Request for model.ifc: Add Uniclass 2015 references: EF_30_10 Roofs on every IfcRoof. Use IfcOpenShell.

First a look at what the model holds.

```python
import ifcopenshell

model = ifcopenshell.open("model.ifc")
print(model.schema)
print("classifications:", [c.Name for c in model.by_type("IfcClassification")])
for ifc_class in ("IfcDoor", "IfcRoof", "IfcStair", "IfcWall", "IfcWindow"):
    print(ifc_class, len(model.by_type(ifc_class)))
```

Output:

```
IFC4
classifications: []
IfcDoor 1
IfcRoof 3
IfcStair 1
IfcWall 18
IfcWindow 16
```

```python
import ifcopenshell
import ifcopenshell.api.classification

model = ifcopenshell.open("model.ifc")

system = ifcopenshell.api.classification.add_classification(model, classification="Uniclass 2015")

codes = {
    "IfcRoof": ("EF_30_10", "Roofs"),
}
for ifc_class, (code, name) in codes.items():
    products = model.by_type(ifc_class)
    ifcopenshell.api.classification.add_reference(
        model, products=products, classification=system, identification=code, name=name
    )
    print(code, len(products))

model.write("model_edited.ifc")
```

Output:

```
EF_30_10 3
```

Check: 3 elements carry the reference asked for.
